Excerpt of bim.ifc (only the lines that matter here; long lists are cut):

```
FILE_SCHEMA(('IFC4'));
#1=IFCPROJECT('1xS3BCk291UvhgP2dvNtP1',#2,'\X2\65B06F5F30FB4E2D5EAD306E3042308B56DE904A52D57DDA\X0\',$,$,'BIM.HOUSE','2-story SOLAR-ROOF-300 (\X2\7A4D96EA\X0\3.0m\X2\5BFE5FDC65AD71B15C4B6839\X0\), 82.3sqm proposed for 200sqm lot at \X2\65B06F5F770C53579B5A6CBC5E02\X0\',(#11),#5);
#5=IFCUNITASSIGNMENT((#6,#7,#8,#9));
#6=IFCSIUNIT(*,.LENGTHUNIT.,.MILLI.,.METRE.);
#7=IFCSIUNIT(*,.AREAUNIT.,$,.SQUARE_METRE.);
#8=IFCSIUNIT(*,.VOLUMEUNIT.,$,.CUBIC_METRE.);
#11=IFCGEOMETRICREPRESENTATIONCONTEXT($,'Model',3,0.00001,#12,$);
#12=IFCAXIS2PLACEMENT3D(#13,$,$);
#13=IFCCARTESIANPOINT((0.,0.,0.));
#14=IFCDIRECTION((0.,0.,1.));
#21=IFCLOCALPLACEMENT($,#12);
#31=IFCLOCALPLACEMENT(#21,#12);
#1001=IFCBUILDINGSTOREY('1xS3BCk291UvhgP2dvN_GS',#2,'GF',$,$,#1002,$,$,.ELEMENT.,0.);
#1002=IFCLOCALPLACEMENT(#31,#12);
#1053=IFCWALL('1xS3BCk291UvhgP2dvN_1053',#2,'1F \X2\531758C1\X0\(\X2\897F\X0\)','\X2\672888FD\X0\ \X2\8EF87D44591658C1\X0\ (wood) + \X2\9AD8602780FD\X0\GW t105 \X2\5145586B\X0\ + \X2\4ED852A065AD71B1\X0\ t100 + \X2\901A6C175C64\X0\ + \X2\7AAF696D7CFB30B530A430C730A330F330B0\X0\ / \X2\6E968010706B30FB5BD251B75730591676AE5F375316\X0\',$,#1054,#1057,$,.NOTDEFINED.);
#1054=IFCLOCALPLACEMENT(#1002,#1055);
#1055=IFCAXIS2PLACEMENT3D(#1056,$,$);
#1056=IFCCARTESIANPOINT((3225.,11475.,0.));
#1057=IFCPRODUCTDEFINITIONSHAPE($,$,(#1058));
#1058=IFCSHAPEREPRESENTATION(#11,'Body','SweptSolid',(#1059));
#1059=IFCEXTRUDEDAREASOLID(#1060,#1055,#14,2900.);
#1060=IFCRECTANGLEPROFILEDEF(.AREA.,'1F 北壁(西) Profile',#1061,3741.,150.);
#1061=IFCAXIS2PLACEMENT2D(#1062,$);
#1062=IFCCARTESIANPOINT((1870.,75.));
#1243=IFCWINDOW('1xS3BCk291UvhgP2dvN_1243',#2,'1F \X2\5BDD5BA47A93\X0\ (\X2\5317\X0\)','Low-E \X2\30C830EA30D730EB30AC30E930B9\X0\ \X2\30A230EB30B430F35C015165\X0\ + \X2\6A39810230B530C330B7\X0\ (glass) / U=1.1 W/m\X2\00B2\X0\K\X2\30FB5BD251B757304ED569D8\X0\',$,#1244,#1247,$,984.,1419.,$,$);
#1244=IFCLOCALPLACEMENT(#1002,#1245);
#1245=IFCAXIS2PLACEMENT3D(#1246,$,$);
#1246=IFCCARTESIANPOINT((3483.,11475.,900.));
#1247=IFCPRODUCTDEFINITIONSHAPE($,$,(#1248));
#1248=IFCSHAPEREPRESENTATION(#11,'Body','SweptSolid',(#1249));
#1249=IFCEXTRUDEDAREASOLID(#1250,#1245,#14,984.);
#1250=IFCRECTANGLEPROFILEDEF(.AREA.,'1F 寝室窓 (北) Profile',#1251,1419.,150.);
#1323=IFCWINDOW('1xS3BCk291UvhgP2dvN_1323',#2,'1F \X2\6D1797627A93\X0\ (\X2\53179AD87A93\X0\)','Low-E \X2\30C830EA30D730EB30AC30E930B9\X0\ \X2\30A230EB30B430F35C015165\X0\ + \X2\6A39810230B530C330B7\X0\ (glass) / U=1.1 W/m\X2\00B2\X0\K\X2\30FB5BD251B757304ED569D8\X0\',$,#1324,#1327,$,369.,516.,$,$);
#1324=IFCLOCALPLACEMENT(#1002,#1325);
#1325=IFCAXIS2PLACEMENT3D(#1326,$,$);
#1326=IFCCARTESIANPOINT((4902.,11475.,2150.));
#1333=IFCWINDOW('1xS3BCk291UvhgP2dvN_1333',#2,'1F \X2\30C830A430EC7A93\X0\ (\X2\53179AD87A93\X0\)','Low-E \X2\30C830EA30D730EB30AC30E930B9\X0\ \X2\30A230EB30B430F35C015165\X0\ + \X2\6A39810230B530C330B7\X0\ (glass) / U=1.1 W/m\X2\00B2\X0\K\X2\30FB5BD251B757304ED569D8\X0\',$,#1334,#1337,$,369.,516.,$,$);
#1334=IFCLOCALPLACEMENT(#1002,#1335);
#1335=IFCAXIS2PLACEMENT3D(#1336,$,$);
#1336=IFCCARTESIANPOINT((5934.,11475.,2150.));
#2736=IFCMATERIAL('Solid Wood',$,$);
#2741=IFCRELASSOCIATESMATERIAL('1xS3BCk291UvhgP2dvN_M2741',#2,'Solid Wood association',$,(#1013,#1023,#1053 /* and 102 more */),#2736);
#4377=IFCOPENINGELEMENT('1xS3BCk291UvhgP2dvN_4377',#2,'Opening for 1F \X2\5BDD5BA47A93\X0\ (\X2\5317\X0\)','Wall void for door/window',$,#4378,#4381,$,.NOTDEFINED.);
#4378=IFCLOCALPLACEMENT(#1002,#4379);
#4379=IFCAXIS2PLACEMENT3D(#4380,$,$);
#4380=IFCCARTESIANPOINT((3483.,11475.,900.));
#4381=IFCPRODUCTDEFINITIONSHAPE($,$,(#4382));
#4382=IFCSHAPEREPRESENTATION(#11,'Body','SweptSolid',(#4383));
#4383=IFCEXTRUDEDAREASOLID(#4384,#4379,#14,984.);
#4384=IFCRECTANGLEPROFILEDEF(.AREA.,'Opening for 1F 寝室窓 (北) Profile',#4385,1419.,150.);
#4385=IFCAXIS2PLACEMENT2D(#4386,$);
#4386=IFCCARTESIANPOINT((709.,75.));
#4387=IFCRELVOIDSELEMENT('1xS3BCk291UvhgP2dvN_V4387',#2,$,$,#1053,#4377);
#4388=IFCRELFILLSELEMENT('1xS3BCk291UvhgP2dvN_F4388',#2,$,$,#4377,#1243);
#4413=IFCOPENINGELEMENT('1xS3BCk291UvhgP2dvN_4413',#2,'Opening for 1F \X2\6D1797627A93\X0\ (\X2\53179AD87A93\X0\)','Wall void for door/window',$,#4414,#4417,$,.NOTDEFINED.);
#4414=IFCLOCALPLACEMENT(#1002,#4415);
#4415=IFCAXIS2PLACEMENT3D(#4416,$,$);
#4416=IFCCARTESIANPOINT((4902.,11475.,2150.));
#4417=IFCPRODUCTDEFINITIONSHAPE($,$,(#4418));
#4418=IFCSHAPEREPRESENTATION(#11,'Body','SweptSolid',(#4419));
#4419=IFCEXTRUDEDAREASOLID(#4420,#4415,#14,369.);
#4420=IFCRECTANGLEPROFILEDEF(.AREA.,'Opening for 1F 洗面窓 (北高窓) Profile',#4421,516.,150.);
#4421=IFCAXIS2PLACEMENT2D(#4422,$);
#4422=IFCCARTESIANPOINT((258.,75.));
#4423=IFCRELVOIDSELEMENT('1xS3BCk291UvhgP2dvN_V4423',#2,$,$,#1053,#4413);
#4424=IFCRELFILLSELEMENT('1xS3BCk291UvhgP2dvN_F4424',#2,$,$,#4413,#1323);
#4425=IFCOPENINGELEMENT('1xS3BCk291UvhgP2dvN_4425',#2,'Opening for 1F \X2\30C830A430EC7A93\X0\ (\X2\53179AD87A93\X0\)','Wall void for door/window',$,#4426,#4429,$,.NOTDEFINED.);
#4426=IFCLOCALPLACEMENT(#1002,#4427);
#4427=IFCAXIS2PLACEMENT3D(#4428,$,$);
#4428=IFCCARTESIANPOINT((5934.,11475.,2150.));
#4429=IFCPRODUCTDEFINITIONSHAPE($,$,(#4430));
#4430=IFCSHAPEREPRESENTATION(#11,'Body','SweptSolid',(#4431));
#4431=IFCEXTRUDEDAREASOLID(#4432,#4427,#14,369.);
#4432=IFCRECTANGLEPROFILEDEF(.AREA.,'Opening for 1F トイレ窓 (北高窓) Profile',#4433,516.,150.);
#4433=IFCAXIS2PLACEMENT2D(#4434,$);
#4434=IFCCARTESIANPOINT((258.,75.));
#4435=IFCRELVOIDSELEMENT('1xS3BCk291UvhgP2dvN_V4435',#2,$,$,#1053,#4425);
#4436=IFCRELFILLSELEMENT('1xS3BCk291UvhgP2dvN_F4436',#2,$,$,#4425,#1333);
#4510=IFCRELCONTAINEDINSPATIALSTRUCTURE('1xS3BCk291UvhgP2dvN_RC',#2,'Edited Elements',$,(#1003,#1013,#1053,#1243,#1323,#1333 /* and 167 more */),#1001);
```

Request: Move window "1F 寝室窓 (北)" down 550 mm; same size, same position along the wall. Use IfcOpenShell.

```python
import numpy as np
import ifcopenshell
import ifcopenshell.api.geometry
import ifcopenshell.util.placement
import ifcopenshell.util.unit

model = ifcopenshell.open("bim.ifc")
unit_scale = ifcopenshell.util.unit.calculate_unit_scale(model)

window = model.by_guid("1xS3BCk291UvhgP2dvN_1243")
opening = window.FillsVoids[0].RelatingOpeningElement
dz = -0.55 / unit_scale

shift = np.array([0.0, 0.0, dz])
# The window is not placed relative to its opening, so move both.
for product in (opening, window):
    matrix = ifcopenshell.util.placement.get_local_placement(product.ObjectPlacement)
    matrix[:3, 3] += shift
    ifcopenshell.api.geometry.edit_object_placement(model, product=product, matrix=matrix, is_si=False)

print(f"moved by {dz * unit_scale:+.3f} m")

model.write("bim_edited.ifc")
```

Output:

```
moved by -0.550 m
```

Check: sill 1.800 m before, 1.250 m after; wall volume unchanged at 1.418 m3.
